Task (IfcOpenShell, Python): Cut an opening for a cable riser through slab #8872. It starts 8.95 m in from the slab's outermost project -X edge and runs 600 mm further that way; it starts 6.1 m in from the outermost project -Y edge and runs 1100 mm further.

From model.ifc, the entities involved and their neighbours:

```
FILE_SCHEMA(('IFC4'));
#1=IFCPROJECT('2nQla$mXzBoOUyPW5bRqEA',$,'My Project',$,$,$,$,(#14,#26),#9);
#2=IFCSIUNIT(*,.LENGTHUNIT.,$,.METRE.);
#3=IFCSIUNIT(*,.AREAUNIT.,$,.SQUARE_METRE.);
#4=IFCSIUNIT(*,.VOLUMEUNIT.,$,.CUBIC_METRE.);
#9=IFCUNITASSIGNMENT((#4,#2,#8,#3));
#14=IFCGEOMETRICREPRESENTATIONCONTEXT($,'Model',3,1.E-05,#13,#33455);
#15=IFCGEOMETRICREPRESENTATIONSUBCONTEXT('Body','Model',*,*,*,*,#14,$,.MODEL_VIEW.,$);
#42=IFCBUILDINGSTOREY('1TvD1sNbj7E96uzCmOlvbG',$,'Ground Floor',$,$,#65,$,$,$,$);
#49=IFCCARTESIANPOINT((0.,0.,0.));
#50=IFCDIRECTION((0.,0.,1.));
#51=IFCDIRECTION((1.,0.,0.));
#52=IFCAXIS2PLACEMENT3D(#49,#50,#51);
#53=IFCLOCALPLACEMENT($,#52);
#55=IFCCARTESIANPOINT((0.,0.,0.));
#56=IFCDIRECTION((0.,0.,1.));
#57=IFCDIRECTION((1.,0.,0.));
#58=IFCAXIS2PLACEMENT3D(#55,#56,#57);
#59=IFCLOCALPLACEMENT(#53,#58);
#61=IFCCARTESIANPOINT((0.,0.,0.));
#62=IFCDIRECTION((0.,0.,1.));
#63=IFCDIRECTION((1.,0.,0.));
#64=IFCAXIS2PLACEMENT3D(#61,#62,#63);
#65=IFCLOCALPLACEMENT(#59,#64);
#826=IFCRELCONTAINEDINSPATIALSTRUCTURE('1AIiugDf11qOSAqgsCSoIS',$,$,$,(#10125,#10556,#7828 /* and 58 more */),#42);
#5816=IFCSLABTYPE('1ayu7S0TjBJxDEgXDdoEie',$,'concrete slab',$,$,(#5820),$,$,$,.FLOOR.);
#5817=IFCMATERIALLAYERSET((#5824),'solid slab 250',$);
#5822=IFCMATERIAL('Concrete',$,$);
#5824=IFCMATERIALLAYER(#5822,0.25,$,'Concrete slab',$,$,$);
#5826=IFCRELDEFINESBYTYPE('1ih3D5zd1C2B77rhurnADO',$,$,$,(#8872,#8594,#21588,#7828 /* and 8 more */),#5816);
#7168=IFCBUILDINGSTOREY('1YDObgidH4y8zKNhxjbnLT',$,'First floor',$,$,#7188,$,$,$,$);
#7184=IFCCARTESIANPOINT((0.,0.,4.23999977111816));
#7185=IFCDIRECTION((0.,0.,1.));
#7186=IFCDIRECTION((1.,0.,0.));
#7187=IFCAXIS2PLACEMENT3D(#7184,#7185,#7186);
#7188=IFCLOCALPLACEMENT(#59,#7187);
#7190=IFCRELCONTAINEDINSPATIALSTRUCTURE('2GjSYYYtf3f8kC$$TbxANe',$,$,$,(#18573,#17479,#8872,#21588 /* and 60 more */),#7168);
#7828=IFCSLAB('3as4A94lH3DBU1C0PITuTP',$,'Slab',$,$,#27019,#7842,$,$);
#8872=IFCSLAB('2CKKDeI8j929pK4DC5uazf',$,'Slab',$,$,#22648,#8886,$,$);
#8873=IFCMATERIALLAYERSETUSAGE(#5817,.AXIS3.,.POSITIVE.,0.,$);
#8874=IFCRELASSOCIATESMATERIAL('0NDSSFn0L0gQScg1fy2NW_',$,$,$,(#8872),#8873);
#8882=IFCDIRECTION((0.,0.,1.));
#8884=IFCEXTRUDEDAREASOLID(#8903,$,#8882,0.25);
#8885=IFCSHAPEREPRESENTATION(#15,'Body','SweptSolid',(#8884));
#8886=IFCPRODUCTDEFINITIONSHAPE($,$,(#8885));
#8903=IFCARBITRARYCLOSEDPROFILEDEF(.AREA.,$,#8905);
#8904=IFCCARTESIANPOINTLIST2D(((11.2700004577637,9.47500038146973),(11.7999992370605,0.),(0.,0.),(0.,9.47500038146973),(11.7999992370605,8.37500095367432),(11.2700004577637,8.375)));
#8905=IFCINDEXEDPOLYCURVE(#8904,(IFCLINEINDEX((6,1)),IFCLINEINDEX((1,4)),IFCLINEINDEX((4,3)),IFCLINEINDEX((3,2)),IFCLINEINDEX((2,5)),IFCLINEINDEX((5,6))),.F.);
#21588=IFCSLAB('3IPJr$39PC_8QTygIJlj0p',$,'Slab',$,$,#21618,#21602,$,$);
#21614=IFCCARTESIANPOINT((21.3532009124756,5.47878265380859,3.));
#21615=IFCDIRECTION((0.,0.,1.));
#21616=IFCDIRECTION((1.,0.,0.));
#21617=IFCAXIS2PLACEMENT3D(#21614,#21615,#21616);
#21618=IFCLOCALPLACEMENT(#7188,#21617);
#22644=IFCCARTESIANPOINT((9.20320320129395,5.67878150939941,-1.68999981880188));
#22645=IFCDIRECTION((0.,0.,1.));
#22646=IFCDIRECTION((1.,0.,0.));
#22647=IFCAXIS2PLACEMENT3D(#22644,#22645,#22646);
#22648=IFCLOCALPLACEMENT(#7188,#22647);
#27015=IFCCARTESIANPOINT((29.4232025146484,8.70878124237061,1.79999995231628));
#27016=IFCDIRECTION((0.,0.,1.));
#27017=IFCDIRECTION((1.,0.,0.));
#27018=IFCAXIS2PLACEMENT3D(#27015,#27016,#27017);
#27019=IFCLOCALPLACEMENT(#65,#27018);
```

```python
import numpy as np
import ifcopenshell
import ifcopenshell.api.feature
import ifcopenshell.api.geometry
import ifcopenshell.api.root
import ifcopenshell.geom
import ifcopenshell.util.placement
import ifcopenshell.util.representation
import ifcopenshell.util.shape
import ifcopenshell.util.unit

model = ifcopenshell.open("model.ifc")
unit_scale = ifcopenshell.util.unit.calculate_unit_scale(model)
settings = ifcopenshell.geom.settings()


def volume(element):
    """Net volume in cubic metres, openings subtracted."""
    shape = ifcopenshell.geom.create_shape(settings, element)
    return ifcopenshell.util.shape.get_volume(shape.geometry)


slab = model.by_guid("2CKKDeI8j929pK4DC5uazf")
before = volume(slab)

# Extent in the slab's own axes, in metres. The edges named are its -X and -Y sides.
slab_shape = ifcopenshell.geom.create_shape(settings, slab)
vertices = ifcopenshell.util.shape.get_vertices(slab_shape.geometry)
x_min, y_min, bottom = vertices.min(axis=0)
top = vertices[:, 2].max()

opening = ifcopenshell.api.root.create_entity(model, ifc_class="IfcOpeningElement", name="Cable riser opening", predefined_type="OPENING")
context = ifcopenshell.util.representation.get_context(model, "Model", "Body", "MODEL_VIEW")
width, depth = 0.6, 1.1
outline = [(0.0, 0.0), (width, 0.0), (width, depth), (0.0, depth), (0.0, 0.0)]
# Overshoot both faces by 50 mm so the cut is clean.
shape = ifcopenshell.api.geometry.add_slab_representation(
    model, context=context, depth=top - bottom + 0.1, polyline=outline
)
ifcopenshell.api.geometry.assign_representation(model, product=opening, representation=shape)

matrix = ifcopenshell.util.placement.get_local_placement(slab.ObjectPlacement)
matrix[:, 3] = matrix @ np.append(np.array([x_min + 8.95, y_min + 6.1, bottom - 0.05]) / unit_scale, 1.0)
ifcopenshell.api.geometry.edit_object_placement(model, product=opening, matrix=matrix, is_si=False)
ifcopenshell.api.feature.add_feature(model, feature=opening, element=slab)

after = volume(slab)

print(f"slab volume {before:.3f} -> {after:.3f} m3")

model.write("model_rev.ifc")
```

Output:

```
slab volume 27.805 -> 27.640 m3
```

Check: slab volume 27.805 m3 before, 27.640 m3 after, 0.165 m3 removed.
